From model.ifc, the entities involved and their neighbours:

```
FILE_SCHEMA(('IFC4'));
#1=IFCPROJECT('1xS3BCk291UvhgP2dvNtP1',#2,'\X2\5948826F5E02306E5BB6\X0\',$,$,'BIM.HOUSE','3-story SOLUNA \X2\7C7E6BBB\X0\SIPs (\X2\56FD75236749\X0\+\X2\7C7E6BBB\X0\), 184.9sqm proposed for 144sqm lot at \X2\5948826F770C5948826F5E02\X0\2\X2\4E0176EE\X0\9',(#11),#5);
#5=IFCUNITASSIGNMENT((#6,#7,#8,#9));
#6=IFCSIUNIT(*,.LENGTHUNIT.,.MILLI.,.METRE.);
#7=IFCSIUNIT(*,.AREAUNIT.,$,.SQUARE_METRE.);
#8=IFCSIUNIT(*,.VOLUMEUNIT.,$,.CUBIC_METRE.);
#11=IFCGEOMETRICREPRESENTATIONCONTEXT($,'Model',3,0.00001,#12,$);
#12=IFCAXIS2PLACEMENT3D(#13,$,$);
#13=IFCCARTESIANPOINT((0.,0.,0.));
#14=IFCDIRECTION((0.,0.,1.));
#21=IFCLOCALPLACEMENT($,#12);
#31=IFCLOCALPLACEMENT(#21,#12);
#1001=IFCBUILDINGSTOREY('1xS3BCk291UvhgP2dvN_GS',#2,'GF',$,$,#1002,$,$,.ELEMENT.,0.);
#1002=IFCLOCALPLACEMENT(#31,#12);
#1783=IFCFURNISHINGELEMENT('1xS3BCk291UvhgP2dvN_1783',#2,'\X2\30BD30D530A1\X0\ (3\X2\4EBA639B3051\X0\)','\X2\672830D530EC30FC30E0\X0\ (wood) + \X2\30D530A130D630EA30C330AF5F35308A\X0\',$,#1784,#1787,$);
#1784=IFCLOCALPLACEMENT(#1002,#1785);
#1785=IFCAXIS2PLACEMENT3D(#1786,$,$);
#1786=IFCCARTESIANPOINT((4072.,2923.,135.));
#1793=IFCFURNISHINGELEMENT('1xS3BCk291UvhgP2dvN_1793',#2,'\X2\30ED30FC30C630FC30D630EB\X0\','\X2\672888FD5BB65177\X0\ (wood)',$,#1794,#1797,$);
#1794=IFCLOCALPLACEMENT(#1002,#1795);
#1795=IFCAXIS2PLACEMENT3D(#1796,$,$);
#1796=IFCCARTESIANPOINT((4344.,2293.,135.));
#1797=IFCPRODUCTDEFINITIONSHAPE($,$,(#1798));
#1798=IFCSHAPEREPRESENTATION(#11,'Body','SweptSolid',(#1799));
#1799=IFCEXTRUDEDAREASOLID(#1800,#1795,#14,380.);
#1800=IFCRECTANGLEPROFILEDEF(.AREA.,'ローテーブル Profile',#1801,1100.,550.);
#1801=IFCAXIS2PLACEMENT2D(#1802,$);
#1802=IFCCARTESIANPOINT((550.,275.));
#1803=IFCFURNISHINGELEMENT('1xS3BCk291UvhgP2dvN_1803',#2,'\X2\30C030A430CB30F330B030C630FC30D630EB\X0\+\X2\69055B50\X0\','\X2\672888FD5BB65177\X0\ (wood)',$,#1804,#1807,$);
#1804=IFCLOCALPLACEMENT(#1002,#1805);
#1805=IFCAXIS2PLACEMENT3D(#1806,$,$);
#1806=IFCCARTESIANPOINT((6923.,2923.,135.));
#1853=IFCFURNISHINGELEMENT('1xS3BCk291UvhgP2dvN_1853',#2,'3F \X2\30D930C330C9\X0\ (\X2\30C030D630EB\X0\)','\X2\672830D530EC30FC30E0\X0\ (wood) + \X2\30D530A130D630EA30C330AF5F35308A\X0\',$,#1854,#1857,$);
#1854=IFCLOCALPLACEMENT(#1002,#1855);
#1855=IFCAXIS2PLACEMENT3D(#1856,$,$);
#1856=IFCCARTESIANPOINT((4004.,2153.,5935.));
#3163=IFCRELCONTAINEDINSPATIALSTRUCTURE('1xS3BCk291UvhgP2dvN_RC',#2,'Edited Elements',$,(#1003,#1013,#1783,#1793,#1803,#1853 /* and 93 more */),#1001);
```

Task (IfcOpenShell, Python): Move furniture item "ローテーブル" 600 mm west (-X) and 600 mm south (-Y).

```python
import ifcopenshell
import ifcopenshell.api.geometry
import ifcopenshell.util.placement
import ifcopenshell.util.unit

model = ifcopenshell.open("model.ifc")
unit_scale = ifcopenshell.util.unit.calculate_unit_scale(model)

item = model.by_guid("1xS3BCk291UvhgP2dvN_1793")
matrix = ifcopenshell.util.placement.get_local_placement(item.ObjectPlacement)
matrix[0, 3] -= 0.6 / unit_scale
matrix[1, 3] -= 0.6 / unit_scale
ifcopenshell.api.geometry.edit_object_placement(model, product=item, matrix=matrix, is_si=False)

print(ifcopenshell.util.placement.get_local_placement(item.ObjectPlacement).round(3) + 0.0)

model.write("model_rev.ifc")
```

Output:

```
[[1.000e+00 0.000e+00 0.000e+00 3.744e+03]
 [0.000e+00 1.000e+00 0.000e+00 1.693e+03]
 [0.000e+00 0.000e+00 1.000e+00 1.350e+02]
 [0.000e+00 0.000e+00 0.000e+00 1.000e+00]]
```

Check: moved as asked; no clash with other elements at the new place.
